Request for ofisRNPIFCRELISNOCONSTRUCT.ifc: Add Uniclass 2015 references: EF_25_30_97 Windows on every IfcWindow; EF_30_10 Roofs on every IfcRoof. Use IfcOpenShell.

First a look at what the model holds.

```python
import ifcopenshell

model = ifcopenshell.open("ofisRNPIFCRELISNOCONSTRUCT.ifc")
print(model.schema)
print("classifications:", [c.Name for c in model.by_type("IfcClassification")])
for ifc_class in ("IfcDoor", "IfcRoof", "IfcStair", "IfcWall", "IfcWindow"):
    print(ifc_class, len(model.by_type(ifc_class)))
```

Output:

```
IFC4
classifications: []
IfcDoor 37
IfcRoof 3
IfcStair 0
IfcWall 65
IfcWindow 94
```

```python
import ifcopenshell
import ifcopenshell.api.classification

model = ifcopenshell.open("ofisRNPIFCRELISNOCONSTRUCT.ifc")

system = ifcopenshell.api.classification.add_classification(model, classification="Uniclass 2015")

codes = {
    "IfcWindow": ("EF_25_30_97", "Windows"),
    "IfcRoof": ("EF_30_10", "Roofs"),
}
for ifc_class, (code, name) in codes.items():
    products = model.by_type(ifc_class)
    ifcopenshell.api.classification.add_reference(
        model, products=products, classification=system, identification=code, name=name
    )
    print(code, len(products))

model.write("ofisRNPIFCRELISNOCONSTRUCT_rev.ifc")
```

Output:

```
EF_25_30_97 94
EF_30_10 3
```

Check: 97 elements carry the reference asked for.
